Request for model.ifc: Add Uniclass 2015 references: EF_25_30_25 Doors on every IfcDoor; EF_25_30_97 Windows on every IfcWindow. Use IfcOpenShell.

First a look at what the model holds.

```python
import ifcopenshell

model = ifcopenshell.open("model.ifc")
print(model.schema)
print("classifications:", [c.Name for c in model.by_type("IfcClassification")])
for ifc_class in ("IfcDoor", "IfcRoof", "IfcStair", "IfcWall", "IfcWindow"):
    print(ifc_class, len(model.by_type(ifc_class)))
```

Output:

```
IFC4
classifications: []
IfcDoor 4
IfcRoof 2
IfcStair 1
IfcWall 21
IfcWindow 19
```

```python
import ifcopenshell
import ifcopenshell.api.classification

model = ifcopenshell.open("model.ifc")

system = ifcopenshell.api.classification.add_classification(model, classification="Uniclass 2015")

codes = {
    "IfcDoor": ("EF_25_30_25", "Doors"),
    "IfcWindow": ("EF_25_30_97", "Windows"),
}
for ifc_class, (code, name) in codes.items():
    products = model.by_type(ifc_class)
    ifcopenshell.api.classification.add_reference(
        model, products=products, classification=system, identification=code, name=name
    )
    print(code, len(products))

model.write("model_v2.ifc")
```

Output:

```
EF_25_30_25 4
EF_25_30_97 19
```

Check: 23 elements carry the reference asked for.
